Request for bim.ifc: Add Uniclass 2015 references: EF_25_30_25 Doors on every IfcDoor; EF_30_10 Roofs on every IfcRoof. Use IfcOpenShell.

First a look at what the model holds.

```python
import ifcopenshell

model = ifcopenshell.open("bim.ifc")
print(model.schema)
print("classifications:", [c.Name for c in model.by_type("IfcClassification")])
for ifc_class in ("IfcDoor", "IfcRoof", "IfcStair", "IfcWall", "IfcWindow"):
    print(ifc_class, len(model.by_type(ifc_class)))
```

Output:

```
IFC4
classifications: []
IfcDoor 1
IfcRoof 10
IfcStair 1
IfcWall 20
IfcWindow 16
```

```python
import ifcopenshell
import ifcopenshell.api.classification

model = ifcopenshell.open("bim.ifc")

system = ifcopenshell.api.classification.add_classification(model, classification="Uniclass 2015")

codes = {
    "IfcDoor": ("EF_25_30_25", "Doors"),
    "IfcRoof": ("EF_30_10", "Roofs"),
}
for ifc_class, (code, name) in codes.items():
    products = model.by_type(ifc_class)
    ifcopenshell.api.classification.add_reference(
        model, products=products, classification=system, identification=code, name=name
    )
    print(code, len(products))

model.write("bim_v2.ifc")
```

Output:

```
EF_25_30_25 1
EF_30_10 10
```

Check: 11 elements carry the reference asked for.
